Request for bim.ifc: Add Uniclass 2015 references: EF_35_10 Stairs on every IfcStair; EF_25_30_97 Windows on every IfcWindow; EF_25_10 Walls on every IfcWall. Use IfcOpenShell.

First a look at what the model holds.

```python
import ifcopenshell

model = ifcopenshell.open("bim.ifc")
print(model.schema)
print("classifications:", [c.Name for c in model.by_type("IfcClassification")])
for ifc_class in ("IfcDoor", "IfcRoof", "IfcStair", "IfcWall", "IfcWindow"):
    print(ifc_class, len(model.by_type(ifc_class)))
```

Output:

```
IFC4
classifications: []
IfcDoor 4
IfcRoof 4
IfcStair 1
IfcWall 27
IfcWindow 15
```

```python
import ifcopenshell
import ifcopenshell.api.classification

model = ifcopenshell.open("bim.ifc")

system = ifcopenshell.api.classification.add_classification(model, classification="Uniclass 2015")

codes = {
    "IfcStair": ("EF_35_10", "Stairs"),
    "IfcWindow": ("EF_25_30_97", "Windows"),
    "IfcWall": ("EF_25_10", "Walls"),
}
for ifc_class, (code, name) in codes.items():
    products = model.by_type(ifc_class)
    ifcopenshell.api.classification.add_reference(
        model, products=products, classification=system, identification=code, name=name
    )
    print(code, len(products))

model.write("bim_updated.ifc")
```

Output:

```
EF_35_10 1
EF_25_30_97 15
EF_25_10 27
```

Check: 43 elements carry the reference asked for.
